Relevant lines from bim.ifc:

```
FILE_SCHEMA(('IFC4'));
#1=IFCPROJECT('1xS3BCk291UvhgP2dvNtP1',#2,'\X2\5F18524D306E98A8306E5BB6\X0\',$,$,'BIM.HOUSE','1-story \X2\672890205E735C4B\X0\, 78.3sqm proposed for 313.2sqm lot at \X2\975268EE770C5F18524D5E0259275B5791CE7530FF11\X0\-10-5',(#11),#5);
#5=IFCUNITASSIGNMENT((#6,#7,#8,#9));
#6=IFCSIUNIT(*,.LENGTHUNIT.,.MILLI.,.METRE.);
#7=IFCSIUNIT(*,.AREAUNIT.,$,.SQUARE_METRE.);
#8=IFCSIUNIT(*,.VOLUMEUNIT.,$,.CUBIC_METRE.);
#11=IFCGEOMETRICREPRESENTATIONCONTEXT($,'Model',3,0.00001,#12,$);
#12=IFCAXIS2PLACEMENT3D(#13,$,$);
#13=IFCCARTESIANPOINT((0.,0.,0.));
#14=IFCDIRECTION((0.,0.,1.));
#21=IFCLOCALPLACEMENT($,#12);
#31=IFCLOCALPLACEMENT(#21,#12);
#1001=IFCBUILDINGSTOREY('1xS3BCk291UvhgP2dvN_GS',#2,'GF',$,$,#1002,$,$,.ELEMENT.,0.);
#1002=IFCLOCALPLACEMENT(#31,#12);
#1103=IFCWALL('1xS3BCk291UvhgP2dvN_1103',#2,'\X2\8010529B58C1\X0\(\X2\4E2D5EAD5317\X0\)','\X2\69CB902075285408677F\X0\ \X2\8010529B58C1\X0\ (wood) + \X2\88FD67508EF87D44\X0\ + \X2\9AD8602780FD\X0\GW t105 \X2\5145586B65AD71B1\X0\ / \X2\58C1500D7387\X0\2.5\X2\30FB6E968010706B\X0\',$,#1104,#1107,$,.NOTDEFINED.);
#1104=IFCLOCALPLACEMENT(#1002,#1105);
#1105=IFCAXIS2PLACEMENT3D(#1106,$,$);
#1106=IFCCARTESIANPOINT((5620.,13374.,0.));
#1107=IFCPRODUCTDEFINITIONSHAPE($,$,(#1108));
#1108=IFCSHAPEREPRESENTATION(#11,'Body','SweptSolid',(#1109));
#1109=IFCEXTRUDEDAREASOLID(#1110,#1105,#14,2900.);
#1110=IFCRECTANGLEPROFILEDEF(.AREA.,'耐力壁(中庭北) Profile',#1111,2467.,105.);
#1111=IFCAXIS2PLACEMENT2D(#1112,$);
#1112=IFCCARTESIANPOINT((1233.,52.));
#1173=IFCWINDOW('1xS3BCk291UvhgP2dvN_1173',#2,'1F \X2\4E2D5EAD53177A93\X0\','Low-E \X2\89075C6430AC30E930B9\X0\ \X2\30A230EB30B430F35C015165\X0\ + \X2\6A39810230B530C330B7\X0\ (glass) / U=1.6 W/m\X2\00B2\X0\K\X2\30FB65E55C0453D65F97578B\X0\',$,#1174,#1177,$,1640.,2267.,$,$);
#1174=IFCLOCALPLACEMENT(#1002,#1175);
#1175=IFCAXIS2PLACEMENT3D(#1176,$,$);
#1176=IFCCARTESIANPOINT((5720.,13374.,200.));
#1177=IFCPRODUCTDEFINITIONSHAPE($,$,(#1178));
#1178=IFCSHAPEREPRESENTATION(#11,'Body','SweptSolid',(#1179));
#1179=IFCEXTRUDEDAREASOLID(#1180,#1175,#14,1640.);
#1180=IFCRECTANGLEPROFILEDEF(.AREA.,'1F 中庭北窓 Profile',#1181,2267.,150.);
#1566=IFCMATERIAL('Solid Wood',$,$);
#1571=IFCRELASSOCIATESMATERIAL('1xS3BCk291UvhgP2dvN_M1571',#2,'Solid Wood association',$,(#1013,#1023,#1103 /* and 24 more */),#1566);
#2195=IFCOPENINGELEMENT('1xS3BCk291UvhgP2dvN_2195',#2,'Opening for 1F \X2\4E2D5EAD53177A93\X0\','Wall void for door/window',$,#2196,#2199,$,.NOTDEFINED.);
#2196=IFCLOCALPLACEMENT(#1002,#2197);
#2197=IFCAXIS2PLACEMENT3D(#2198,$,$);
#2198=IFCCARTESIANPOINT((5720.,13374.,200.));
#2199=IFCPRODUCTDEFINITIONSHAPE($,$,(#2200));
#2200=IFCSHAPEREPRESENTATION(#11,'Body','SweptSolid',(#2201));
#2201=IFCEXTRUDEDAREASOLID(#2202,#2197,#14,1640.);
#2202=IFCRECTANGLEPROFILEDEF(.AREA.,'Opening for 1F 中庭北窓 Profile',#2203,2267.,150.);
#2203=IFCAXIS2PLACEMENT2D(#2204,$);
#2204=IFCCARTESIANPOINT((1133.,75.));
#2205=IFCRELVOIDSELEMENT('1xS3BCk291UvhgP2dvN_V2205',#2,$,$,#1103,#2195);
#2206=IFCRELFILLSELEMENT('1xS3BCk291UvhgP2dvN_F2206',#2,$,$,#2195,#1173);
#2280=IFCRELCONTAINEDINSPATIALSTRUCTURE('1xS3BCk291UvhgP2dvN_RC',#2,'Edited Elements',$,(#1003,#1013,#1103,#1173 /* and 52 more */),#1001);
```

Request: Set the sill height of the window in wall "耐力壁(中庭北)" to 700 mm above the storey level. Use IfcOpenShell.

```python
import numpy as np
import ifcopenshell
import ifcopenshell.api.geometry
import ifcopenshell.geom
import ifcopenshell.util.element
import ifcopenshell.util.placement
import ifcopenshell.util.shape
import ifcopenshell.util.unit

model = ifcopenshell.open("bim.ifc")
unit_scale = ifcopenshell.util.unit.calculate_unit_scale(model)

window = model.by_id(1173)
opening = window.FillsVoids[0].RelatingOpeningElement
storey = ifcopenshell.util.element.get_container(window, ifc_class="IfcBuildingStorey")
level = ifcopenshell.util.placement.get_local_placement(storey.ObjectPlacement)[2, 3]

# The opening's origin need not be at the sill, so measure its lowest point.
shape = ifcopenshell.geom.create_shape(ifcopenshell.geom.settings(), opening)
bottom = ifcopenshell.util.shape.get_shape_bottom_elevation(shape, shape.geometry) / unit_scale
dz = level + 0.7 / unit_scale - bottom

shift = np.array([0.0, 0.0, dz])
# The window is not placed relative to its opening, so move both.
for product in (opening, window):
    matrix = ifcopenshell.util.placement.get_local_placement(product.ObjectPlacement)
    matrix[:3, 3] += shift
    ifcopenshell.api.geometry.edit_object_placement(model, product=product, matrix=matrix, is_si=False)

print(f"moved by {dz * unit_scale:+.3f} m")

model.write("bim_rev.ifc")
```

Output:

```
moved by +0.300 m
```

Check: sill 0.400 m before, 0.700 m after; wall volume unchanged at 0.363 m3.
